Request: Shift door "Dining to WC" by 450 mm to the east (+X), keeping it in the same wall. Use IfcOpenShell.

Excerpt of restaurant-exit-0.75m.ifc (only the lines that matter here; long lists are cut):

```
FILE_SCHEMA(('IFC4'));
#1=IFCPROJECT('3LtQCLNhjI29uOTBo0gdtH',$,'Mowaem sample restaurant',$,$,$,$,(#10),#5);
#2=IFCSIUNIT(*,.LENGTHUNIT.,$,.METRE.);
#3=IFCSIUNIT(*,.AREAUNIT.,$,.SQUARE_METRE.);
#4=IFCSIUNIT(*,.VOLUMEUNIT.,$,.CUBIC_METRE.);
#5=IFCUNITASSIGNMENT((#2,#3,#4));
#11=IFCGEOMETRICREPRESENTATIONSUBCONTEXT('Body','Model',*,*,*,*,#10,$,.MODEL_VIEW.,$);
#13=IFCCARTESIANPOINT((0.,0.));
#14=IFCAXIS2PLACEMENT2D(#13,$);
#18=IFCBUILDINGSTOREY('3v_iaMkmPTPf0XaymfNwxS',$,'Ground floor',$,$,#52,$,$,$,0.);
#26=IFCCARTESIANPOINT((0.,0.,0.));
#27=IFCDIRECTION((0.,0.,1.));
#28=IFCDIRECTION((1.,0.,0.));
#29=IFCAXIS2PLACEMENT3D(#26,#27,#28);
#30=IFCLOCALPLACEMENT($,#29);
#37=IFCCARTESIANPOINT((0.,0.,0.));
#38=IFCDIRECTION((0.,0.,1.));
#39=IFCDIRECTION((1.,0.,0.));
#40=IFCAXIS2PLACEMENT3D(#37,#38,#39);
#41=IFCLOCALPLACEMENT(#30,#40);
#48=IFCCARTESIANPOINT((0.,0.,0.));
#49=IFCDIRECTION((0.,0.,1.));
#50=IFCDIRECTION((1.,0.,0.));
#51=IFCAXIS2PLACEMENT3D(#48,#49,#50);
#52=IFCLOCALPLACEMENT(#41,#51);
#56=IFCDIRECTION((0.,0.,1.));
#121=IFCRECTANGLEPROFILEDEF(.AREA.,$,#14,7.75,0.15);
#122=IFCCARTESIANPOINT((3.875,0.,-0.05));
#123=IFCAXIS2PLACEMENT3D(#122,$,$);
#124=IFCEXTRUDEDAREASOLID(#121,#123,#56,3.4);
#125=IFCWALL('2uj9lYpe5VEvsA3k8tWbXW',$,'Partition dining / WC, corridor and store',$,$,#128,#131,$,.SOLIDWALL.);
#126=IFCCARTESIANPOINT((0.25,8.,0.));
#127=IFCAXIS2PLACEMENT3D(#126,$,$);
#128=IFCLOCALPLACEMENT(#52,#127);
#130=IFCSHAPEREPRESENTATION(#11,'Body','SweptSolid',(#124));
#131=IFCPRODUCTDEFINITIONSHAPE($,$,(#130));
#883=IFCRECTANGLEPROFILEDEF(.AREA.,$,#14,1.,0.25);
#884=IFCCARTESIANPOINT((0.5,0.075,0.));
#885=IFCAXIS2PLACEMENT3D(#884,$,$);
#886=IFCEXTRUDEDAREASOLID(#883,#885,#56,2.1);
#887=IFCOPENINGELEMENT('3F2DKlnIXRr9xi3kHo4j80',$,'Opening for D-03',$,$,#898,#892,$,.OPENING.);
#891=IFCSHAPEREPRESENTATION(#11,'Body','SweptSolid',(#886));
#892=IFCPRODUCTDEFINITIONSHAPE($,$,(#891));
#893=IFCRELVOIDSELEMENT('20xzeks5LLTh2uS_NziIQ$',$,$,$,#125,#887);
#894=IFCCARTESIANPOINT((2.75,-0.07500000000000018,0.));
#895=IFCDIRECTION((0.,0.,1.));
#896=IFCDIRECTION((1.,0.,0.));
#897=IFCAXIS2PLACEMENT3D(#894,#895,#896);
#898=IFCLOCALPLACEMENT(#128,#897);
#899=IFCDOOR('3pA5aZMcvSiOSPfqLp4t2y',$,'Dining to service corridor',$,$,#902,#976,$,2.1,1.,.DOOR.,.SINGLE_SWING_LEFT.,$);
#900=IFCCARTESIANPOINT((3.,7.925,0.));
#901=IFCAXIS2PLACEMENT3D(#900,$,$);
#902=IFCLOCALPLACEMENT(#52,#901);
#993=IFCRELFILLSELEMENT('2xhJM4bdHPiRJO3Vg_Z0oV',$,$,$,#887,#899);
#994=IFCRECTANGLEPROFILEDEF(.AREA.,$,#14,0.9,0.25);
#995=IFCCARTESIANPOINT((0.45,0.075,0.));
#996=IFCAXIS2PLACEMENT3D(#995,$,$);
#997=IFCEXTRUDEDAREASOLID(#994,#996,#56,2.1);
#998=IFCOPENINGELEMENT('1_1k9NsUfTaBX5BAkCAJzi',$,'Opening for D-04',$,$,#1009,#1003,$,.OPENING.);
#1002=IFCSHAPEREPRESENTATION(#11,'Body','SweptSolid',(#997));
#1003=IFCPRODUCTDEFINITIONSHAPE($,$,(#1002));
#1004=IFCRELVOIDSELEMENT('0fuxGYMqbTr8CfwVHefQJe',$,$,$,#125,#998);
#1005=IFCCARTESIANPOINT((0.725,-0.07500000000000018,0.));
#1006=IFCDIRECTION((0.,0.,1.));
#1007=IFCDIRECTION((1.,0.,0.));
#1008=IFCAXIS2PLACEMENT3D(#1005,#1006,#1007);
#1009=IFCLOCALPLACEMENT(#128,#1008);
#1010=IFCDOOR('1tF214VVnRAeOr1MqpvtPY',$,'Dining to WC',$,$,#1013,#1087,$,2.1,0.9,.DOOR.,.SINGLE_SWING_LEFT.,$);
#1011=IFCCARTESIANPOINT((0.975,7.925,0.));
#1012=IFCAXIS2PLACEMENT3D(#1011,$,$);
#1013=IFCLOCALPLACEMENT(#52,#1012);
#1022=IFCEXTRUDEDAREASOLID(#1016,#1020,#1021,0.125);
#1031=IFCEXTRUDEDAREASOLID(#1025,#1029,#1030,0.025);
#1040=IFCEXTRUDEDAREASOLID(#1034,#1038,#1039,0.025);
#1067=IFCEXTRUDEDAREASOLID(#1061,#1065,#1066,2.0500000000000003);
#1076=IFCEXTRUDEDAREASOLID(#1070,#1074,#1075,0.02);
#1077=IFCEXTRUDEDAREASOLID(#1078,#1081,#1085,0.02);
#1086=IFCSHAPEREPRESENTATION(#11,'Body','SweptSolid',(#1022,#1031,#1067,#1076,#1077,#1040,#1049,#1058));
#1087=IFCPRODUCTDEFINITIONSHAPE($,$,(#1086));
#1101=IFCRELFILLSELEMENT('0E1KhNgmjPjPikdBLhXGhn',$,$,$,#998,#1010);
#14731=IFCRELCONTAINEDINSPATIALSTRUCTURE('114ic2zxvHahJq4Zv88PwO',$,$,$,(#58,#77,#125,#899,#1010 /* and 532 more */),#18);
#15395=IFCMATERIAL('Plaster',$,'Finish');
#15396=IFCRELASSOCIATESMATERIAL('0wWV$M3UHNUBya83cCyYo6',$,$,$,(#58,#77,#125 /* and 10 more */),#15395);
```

```python
import ifcopenshell
import ifcopenshell.api.geometry
import ifcopenshell.util.placement

model = ifcopenshell.open("restaurant-exit-0.75m.ifc")

door = model.by_guid("1tF214VVnRAeOr1MqpvtPY")
opening = door.FillsVoids[0].RelatingOpeningElement
wall = opening.VoidsElements[0].RelatingBuildingElement

wall_matrix = ifcopenshell.util.placement.get_local_placement(wall.ObjectPlacement)
shift = wall_matrix[:3, 0] * 0.45
before = ifcopenshell.util.placement.get_local_placement(door.ObjectPlacement)[:3, 3].copy()

# The door is not placed relative to its opening, so move both.
for product in (opening, door):
    matrix = ifcopenshell.util.placement.get_local_placement(product.ObjectPlacement)
    matrix[:3, 3] += shift
    ifcopenshell.api.geometry.edit_object_placement(model, product=product, matrix=matrix, is_si=False)

after = ifcopenshell.util.placement.get_local_placement(door.ObjectPlacement)[:3, 3]
print("door moved by", (after - before).round(3) + 0.0)

model.write("restaurant-exit-0.75m_edited.ifc")
```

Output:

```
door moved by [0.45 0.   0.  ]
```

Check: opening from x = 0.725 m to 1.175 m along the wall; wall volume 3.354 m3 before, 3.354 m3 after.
